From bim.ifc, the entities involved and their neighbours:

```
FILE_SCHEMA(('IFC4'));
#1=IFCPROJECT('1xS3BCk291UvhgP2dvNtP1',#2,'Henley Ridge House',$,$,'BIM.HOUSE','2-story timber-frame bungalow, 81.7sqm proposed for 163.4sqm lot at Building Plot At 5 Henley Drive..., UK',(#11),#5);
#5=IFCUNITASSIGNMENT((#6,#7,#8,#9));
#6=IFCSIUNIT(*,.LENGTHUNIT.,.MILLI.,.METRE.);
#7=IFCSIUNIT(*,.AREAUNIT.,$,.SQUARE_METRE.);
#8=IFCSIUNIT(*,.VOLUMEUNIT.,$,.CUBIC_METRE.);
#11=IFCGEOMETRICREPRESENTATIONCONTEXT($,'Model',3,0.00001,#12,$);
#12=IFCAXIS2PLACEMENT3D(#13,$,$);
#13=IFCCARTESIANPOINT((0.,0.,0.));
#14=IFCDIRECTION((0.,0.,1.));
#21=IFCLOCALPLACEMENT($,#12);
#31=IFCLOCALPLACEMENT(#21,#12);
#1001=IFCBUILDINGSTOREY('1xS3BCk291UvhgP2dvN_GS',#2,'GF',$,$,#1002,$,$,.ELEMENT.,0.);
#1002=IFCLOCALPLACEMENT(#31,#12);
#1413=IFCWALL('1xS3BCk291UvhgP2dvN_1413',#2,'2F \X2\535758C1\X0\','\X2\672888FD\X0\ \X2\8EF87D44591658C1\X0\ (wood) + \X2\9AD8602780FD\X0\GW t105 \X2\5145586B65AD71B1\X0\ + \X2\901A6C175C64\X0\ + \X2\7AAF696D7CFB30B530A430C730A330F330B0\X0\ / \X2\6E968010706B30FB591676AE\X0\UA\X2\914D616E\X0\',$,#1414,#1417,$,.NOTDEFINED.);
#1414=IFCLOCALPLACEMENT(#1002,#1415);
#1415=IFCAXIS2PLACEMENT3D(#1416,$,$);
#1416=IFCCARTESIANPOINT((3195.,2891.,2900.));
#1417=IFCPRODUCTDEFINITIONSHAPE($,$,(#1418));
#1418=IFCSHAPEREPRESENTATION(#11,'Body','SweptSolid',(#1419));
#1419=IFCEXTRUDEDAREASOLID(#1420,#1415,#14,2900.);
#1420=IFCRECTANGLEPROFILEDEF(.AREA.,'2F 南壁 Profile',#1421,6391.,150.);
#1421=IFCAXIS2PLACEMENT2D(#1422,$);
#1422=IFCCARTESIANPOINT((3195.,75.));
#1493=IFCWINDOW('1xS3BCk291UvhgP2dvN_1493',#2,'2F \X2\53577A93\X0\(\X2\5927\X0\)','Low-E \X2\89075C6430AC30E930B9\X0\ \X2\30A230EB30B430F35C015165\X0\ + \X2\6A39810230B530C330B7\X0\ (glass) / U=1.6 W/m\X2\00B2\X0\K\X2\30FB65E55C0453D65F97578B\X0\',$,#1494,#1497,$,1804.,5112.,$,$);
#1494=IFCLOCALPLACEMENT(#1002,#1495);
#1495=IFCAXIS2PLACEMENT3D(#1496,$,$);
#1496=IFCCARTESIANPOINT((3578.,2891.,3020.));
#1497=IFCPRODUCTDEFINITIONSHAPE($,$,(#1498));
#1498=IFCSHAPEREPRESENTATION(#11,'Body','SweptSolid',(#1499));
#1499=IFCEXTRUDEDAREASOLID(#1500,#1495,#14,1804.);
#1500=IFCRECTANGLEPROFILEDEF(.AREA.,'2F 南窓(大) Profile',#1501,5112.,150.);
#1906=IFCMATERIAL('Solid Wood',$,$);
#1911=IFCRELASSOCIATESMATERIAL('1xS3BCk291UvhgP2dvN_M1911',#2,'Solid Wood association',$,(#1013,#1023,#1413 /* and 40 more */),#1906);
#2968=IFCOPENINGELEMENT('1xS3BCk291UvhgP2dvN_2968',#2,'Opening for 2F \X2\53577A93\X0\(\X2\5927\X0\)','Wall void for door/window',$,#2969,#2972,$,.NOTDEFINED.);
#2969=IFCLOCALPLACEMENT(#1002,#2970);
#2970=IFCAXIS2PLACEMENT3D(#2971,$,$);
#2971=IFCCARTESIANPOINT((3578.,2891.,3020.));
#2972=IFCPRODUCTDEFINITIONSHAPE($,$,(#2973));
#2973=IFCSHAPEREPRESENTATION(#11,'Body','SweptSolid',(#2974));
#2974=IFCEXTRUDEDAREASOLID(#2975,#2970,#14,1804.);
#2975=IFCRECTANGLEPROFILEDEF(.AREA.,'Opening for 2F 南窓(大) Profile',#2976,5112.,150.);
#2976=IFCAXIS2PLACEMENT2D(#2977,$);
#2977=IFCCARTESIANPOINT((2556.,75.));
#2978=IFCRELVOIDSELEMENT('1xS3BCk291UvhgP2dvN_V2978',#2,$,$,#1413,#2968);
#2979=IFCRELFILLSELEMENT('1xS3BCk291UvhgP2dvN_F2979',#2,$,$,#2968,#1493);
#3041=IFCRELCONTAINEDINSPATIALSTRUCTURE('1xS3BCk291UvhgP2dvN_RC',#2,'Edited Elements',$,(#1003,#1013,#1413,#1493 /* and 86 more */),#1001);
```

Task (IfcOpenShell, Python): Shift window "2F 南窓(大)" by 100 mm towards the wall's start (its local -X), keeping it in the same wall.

```python
import ifcopenshell
import ifcopenshell.api.geometry
import ifcopenshell.util.placement
import ifcopenshell.util.unit

model = ifcopenshell.open("bim.ifc")
unit_scale = ifcopenshell.util.unit.calculate_unit_scale(model)

window = model.by_guid("1xS3BCk291UvhgP2dvN_1493")
opening = window.FillsVoids[0].RelatingOpeningElement
wall = opening.VoidsElements[0].RelatingBuildingElement

wall_matrix = ifcopenshell.util.placement.get_local_placement(wall.ObjectPlacement)
shift = wall_matrix[:3, 0] * -0.1 / unit_scale
before = ifcopenshell.util.placement.get_local_placement(window.ObjectPlacement)[:3, 3].copy()

# The window is not placed relative to its opening, so move both.
for product in (opening, window):
    matrix = ifcopenshell.util.placement.get_local_placement(product.ObjectPlacement)
    matrix[:3, 3] += shift
    ifcopenshell.api.geometry.edit_object_placement(model, product=product, matrix=matrix, is_si=False)

after = ifcopenshell.util.placement.get_local_placement(window.ObjectPlacement)[:3, 3]
print("window moved by", (after - before).round(3) + 0.0)

model.write("bim_rev.ifc")
```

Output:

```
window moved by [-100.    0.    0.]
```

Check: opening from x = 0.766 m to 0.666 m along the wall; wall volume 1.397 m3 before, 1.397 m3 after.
